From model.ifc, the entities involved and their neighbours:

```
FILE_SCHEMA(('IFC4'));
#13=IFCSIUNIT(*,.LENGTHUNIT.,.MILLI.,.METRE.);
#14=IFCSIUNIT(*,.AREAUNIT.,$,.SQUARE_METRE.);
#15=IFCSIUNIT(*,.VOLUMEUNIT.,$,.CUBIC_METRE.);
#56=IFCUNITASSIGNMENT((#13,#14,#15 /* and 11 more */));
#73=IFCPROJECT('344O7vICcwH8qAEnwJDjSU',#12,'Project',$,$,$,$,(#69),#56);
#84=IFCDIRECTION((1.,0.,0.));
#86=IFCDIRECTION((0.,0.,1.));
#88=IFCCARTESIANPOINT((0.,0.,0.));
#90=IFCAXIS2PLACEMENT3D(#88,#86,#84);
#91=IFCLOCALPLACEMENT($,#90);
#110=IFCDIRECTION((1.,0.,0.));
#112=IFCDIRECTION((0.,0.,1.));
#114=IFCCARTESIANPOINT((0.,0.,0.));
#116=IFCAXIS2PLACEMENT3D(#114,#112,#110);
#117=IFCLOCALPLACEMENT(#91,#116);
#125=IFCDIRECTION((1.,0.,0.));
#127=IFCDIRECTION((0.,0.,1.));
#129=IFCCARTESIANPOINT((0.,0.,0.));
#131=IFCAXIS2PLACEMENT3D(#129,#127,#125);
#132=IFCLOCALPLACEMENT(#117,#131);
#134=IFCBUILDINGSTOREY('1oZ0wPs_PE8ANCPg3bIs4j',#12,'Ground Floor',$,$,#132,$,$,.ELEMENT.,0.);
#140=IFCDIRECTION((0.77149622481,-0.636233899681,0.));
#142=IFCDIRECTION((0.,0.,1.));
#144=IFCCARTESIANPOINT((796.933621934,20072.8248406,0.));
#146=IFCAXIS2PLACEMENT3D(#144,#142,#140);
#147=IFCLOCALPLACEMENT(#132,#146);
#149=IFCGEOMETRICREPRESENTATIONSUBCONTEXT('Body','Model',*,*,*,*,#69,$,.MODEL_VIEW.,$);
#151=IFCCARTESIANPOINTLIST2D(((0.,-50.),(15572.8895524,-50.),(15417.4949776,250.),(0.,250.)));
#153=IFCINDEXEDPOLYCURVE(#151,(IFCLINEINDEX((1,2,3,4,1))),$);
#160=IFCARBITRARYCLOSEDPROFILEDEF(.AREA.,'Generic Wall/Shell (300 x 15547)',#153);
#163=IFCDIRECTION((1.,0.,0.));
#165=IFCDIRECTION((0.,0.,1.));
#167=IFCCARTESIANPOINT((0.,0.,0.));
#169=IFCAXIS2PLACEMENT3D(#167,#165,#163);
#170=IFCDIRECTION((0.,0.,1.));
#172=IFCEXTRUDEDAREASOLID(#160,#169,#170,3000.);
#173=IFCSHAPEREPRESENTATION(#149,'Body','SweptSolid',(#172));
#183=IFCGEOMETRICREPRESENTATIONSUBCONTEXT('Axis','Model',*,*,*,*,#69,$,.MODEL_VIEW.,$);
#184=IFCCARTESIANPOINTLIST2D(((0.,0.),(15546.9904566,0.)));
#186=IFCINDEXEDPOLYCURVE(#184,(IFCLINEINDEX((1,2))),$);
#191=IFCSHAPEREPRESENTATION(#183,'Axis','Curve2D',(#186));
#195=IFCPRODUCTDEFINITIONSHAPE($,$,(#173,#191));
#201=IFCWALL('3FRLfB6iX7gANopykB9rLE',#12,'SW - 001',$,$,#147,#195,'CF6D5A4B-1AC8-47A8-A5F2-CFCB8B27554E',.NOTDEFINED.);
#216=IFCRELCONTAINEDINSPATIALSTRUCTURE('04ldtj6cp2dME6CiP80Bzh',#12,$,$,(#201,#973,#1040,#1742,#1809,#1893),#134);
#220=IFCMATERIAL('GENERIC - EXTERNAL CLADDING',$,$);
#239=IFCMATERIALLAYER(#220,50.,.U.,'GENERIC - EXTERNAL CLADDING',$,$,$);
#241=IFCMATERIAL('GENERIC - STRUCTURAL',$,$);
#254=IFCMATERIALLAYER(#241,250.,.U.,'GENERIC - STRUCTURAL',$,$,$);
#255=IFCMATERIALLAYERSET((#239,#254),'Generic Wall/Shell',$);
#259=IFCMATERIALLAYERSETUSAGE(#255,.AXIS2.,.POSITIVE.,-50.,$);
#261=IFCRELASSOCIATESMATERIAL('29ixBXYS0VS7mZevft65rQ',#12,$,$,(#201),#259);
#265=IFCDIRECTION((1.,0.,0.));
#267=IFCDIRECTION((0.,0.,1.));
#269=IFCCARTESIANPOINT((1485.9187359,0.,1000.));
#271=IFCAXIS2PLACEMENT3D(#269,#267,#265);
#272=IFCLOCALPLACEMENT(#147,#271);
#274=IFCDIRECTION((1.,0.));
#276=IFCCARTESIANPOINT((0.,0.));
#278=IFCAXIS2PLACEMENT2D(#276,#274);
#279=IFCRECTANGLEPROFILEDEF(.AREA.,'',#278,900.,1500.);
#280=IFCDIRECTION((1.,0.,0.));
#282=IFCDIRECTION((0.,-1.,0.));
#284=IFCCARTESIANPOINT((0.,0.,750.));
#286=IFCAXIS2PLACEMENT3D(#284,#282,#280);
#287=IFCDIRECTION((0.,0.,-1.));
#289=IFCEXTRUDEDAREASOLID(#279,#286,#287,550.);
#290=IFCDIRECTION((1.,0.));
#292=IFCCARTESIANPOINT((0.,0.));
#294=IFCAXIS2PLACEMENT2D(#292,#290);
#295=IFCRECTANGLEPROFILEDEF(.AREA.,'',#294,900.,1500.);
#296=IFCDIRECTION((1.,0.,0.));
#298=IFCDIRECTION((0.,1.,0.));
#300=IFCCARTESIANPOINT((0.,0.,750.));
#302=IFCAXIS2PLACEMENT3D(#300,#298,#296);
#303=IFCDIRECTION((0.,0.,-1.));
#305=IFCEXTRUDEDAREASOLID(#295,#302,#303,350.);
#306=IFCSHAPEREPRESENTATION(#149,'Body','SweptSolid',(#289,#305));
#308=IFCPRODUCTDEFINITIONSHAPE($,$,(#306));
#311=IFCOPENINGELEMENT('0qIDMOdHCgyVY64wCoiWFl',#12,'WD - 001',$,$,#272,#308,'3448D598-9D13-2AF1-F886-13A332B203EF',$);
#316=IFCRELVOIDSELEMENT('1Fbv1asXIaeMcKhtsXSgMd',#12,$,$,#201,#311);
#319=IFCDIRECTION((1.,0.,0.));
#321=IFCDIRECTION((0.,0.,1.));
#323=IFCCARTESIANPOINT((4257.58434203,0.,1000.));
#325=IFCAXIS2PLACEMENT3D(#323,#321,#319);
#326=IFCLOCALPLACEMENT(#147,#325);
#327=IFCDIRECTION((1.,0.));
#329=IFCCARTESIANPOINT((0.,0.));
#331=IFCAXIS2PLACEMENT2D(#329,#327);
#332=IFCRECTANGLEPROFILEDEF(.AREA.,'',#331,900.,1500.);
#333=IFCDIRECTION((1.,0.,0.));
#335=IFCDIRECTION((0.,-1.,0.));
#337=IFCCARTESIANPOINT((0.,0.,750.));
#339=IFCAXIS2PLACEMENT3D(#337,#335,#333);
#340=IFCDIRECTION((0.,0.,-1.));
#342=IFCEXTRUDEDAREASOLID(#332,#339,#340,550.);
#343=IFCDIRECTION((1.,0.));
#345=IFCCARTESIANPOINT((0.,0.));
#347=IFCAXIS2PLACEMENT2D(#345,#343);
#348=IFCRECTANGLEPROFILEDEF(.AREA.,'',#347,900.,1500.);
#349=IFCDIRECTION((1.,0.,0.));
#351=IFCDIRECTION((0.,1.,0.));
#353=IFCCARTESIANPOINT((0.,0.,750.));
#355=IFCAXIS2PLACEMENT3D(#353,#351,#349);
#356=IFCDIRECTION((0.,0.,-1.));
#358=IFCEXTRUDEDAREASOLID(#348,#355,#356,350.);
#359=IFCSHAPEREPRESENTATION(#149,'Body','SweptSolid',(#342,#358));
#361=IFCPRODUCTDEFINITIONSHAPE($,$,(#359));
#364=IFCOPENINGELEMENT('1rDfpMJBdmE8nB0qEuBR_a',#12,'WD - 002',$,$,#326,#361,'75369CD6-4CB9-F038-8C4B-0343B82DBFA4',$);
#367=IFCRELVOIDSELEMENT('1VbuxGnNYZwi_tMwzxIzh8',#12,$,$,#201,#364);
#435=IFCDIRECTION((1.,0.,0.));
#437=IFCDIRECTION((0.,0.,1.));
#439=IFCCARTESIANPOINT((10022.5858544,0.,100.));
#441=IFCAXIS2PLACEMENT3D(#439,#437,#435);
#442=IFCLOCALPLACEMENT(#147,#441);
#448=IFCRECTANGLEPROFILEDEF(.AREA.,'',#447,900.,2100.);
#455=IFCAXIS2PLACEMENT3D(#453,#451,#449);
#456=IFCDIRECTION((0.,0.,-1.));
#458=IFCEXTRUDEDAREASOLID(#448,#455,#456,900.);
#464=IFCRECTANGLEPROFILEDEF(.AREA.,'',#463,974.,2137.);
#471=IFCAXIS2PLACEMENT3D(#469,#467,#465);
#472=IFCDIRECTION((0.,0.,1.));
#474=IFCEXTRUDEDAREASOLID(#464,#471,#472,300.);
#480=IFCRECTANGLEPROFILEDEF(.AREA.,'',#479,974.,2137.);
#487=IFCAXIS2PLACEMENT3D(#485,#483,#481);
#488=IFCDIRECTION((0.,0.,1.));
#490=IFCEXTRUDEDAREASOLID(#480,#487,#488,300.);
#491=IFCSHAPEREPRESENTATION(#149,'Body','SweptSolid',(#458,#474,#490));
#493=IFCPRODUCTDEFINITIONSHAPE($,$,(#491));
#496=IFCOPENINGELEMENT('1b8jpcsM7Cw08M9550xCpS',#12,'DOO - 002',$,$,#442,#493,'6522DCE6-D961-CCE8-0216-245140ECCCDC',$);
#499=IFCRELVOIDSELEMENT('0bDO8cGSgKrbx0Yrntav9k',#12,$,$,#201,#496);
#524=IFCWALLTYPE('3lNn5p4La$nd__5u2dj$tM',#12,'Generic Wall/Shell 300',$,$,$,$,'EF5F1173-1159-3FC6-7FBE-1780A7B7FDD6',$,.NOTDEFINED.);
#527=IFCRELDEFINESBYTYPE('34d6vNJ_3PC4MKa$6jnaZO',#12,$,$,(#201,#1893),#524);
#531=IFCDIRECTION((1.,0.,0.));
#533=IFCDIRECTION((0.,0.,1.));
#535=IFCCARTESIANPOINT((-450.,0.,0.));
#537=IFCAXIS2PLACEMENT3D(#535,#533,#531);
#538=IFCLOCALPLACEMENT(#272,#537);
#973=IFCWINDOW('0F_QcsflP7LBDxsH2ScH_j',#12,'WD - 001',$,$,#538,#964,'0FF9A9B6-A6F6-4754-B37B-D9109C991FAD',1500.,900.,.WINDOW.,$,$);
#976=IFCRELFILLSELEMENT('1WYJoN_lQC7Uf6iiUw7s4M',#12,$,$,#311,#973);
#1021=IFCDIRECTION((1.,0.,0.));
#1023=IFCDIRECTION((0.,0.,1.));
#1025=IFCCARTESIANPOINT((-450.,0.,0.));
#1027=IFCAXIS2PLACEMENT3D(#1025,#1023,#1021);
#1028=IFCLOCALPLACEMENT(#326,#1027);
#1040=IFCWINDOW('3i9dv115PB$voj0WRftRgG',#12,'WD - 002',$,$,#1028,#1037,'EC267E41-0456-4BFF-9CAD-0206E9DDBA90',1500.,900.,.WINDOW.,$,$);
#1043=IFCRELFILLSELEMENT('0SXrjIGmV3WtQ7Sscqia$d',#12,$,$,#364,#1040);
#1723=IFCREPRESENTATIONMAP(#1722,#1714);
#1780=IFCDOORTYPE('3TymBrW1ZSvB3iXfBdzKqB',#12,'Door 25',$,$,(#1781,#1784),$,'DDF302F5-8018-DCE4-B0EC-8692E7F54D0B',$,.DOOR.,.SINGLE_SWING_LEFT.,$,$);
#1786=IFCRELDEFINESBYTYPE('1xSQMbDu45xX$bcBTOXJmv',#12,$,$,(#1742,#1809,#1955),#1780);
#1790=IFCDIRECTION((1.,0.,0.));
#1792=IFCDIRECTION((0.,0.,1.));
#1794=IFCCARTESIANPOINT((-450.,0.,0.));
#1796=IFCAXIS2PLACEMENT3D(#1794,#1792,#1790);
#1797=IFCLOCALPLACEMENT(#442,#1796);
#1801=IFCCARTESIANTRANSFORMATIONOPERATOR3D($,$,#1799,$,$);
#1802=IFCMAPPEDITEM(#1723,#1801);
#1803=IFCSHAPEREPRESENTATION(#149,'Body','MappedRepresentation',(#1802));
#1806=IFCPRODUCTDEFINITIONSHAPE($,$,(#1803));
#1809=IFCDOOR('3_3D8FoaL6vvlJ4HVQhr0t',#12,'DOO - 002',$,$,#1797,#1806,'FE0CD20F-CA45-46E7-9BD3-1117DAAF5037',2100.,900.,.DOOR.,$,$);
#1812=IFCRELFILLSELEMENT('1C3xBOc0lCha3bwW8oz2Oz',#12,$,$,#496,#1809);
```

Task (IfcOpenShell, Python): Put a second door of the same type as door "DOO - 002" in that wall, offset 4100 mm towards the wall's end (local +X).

```python
import ifcopenshell
import ifcopenshell.api.feature
import ifcopenshell.api.geometry
import ifcopenshell.api.root
import ifcopenshell.geom
import ifcopenshell.util.element
import ifcopenshell.util.placement
import ifcopenshell.util.shape

model = ifcopenshell.open("model.ifc")
settings = ifcopenshell.geom.settings()


def volume(element):
    """Net volume in cubic metres, openings subtracted."""
    shape = ifcopenshell.geom.create_shape(settings, element)
    return ifcopenshell.util.shape.get_volume(shape.geometry)


def reuse_history(source, copy):
    """copy_class also copies each property set's owner history, people and application; keep the originals."""
    for rel in copy.IsDefinedBy:
        if rel.is_a("IfcRelDefinesByProperties") and (history := rel.RelatingPropertyDefinition.OwnerHistory):
            rel.RelatingPropertyDefinition.OwnerHistory = source.OwnerHistory
            ifcopenshell.util.element.remove_deep2(model, history)


door = model.by_id(1809)
opening = door.FillsVoids[0].RelatingOpeningElement
wall = opening.VoidsElements[0].RelatingBuildingElement
before = volume(wall)
shift = ifcopenshell.util.placement.get_local_placement(wall.ObjectPlacement)[:3, 0] * 4100.0

# copy_class copies the void relationship, type, container and properties, but no geometry.
new_opening = ifcopenshell.api.root.copy_class(model, product=opening)
new_opening.Representation = ifcopenshell.util.element.copy_deep(
    model, opening.Representation, exclude=["IfcGeometricRepresentationContext", "IfcRepresentationMap"]
)
new_opening.Tag = None
new_door = ifcopenshell.api.root.copy_class(model, product=door)
new_door.Representation = ifcopenshell.util.element.copy_deep(
    model, door.Representation, exclude=["IfcGeometricRepresentationContext", "IfcRepresentationMap"]
)
new_door.Tag = None
reuse_history(door, new_door)
ifcopenshell.api.feature.add_filling(model, opening=new_opening, element=new_door)

for old, new in ((opening, new_opening), (door, new_door)):
    matrix = ifcopenshell.util.placement.get_local_placement(old.ObjectPlacement)
    matrix[:3, 3] += shift
    ifcopenshell.api.geometry.edit_object_placement(model, product=new, matrix=matrix, is_si=False)

after = volume(wall)

print(f"wall volume {before:.3f} -> {after:.3f} m3")

model.write("model-out.ifc")
```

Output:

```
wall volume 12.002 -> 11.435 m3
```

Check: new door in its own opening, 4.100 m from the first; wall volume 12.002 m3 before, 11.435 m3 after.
